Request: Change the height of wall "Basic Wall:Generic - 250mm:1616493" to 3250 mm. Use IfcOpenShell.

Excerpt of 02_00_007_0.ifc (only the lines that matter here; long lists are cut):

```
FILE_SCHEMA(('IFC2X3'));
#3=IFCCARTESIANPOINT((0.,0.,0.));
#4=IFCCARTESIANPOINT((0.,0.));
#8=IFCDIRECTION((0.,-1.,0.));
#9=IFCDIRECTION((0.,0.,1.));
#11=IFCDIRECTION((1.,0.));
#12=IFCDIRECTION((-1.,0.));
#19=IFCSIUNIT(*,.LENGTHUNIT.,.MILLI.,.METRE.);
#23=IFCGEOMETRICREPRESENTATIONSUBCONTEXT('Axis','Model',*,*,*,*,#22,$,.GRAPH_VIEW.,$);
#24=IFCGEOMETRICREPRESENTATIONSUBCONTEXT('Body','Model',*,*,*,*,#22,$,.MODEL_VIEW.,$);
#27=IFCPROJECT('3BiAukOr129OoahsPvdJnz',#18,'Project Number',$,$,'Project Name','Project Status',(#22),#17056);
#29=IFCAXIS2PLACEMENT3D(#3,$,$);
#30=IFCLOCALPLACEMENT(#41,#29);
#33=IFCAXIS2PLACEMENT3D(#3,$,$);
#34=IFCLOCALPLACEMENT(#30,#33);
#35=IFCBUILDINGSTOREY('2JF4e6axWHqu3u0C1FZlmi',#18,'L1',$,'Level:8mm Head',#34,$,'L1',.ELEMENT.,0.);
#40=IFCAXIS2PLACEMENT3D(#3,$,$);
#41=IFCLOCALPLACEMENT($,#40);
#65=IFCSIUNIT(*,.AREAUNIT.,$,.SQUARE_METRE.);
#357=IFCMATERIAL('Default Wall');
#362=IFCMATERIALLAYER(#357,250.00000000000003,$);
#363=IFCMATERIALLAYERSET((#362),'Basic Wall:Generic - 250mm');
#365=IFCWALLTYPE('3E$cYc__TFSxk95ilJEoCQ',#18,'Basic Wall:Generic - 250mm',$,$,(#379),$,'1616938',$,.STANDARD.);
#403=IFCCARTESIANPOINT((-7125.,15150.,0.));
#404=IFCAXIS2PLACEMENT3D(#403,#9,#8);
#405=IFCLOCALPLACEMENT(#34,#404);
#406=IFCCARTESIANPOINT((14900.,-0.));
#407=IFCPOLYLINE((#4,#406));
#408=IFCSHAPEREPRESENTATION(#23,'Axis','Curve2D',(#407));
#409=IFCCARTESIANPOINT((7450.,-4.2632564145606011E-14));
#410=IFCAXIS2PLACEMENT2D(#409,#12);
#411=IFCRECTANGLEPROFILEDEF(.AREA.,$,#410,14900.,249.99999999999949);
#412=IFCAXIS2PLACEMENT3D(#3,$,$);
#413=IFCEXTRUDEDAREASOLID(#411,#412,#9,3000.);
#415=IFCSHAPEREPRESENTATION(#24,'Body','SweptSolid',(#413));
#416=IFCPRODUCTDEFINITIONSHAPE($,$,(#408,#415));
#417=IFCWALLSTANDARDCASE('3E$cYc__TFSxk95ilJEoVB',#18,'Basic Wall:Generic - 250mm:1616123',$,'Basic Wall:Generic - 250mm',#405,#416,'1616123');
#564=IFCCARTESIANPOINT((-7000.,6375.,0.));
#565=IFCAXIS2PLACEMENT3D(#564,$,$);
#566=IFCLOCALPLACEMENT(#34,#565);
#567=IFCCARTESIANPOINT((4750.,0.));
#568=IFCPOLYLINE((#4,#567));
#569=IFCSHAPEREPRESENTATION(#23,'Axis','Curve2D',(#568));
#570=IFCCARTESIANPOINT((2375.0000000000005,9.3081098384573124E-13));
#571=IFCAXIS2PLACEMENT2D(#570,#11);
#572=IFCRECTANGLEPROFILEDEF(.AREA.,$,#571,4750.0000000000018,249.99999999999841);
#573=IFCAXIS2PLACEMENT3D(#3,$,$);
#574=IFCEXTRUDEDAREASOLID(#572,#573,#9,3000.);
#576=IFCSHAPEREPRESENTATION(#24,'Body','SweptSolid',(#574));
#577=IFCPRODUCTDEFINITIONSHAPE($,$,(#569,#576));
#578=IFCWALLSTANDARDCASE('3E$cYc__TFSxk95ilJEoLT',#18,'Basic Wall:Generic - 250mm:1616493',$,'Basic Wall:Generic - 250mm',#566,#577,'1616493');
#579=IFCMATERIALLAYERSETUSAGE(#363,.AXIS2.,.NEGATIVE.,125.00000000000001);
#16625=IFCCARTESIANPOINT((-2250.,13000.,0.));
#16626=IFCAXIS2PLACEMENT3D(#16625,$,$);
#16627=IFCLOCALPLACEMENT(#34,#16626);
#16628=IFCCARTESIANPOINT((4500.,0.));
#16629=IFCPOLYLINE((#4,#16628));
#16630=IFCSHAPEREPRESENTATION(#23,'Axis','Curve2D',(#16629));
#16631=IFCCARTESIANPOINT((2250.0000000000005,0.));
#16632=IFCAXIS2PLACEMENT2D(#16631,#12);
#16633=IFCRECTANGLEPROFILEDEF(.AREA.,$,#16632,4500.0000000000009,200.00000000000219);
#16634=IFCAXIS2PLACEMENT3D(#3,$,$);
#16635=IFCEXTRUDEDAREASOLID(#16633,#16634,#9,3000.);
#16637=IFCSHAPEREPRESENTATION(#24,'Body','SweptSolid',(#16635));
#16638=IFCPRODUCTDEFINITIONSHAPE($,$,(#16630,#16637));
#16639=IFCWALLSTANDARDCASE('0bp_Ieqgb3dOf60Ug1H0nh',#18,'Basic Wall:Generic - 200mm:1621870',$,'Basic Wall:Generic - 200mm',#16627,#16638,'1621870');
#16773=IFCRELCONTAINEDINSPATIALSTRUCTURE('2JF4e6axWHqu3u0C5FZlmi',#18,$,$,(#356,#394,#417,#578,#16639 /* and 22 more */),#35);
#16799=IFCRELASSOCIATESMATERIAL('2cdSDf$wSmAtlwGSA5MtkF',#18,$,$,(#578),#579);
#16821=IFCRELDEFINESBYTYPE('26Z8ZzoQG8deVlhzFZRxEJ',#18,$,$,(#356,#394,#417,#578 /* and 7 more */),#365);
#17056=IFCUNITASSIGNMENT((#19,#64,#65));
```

```python
import ifcopenshell
import ifcopenshell.geom
import ifcopenshell.util.representation
import ifcopenshell.util.shape
import ifcopenshell.util.unit

model = ifcopenshell.open("02_00_007_0.ifc")
unit_scale = ifcopenshell.util.unit.calculate_unit_scale(model)
settings = ifcopenshell.geom.settings()


def volume(element):
    """Net volume in cubic metres, openings subtracted."""
    shape = ifcopenshell.geom.create_shape(settings, element)
    return ifcopenshell.util.shape.get_volume(shape.geometry)


wall = model.by_guid("3E$cYc__TFSxk95ilJEoLT")
before = volume(wall)

body = ifcopenshell.util.representation.get_representation(wall, "Model", "Body")
solid = body.Items[0]
old_height = solid.Depth
solid.Depth = 3.25 / unit_scale
after = volume(wall)

print(f"height {old_height:g} -> {solid.Depth:g}, volume {before:.3f} -> {after:.3f} m3")

model.write("02_00_007_0_rev.ifc")
```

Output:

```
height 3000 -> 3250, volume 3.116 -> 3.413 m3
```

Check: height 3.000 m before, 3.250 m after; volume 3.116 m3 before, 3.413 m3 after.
